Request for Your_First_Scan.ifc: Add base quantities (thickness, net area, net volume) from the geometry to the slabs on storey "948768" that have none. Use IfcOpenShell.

First a look at what the model holds.

```python
import ifcopenshell
import ifcopenshell.util.element
import ifcopenshell.util.unit

model = ifcopenshell.open("Your_First_Scan.ifc")
print(model.schema)
for unit_type in ("LENGTHUNIT", "AREAUNIT", "VOLUMEUNIT"):
    print(unit_type, ifcopenshell.util.unit.calculate_unit_scale(model, unit_type))
storey = next(s for s in model.by_type("IfcBuildingStorey") if s.Name == "948768")
slabs = [e for e in ifcopenshell.util.element.get_decomposition(storey) if e.is_a("IfcSlab")]
for e in sorted(slabs, key=lambda e: e.id()):
    print(e.id(), e.is_a(), e.Name, list(ifcopenshell.util.element.get_psets(e, qtos_only=True)), sep=" | ")
```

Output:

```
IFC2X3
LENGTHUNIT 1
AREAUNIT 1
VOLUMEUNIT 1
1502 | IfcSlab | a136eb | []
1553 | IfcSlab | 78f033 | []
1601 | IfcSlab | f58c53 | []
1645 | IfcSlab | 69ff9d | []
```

```python
import ifcopenshell
import ifcopenshell.api.pset
import ifcopenshell.geom
import ifcopenshell.util.element
import ifcopenshell.util.shape
import ifcopenshell.util.unit

model = ifcopenshell.open("Your_First_Scan.ifc")
unit_scale = ifcopenshell.util.unit.calculate_unit_scale(model)
area_scale = ifcopenshell.util.unit.calculate_unit_scale(model, "AREAUNIT")
volume_scale = ifcopenshell.util.unit.calculate_unit_scale(model, "VOLUMEUNIT")
settings = ifcopenshell.geom.settings()

storey = next(s for s in model.by_type("IfcBuildingStorey") if s.Name == "948768")
slabs = [e for e in ifcopenshell.util.element.get_decomposition(storey) if e.is_a("IfcSlab")]

for e in sorted(slabs, key=lambda e: e.id()):
    if ifcopenshell.util.element.get_psets(e, qtos_only=True, should_inherit=False):
        continue
    # Geometry comes back in metres, in the element's own axes.
    shape = ifcopenshell.geom.create_shape(settings, e)
    values = {
        "Width": ifcopenshell.util.shape.get_z(shape.geometry) / unit_scale,
        "NetArea": ifcopenshell.util.shape.get_footprint_area(shape.geometry) / area_scale,
        "NetVolume": ifcopenshell.util.shape.get_volume(shape.geometry) / volume_scale,
    }
    qto = ifcopenshell.api.pset.add_qto(model, product=e, name="BaseQuantities")
    ifcopenshell.api.pset.edit_qto(model, qto=qto, properties=values)
    print(e.id(), {k: round(v, 3) for k, v in values.items()})

model.write("Your_First_Scan_rev.ifc")
```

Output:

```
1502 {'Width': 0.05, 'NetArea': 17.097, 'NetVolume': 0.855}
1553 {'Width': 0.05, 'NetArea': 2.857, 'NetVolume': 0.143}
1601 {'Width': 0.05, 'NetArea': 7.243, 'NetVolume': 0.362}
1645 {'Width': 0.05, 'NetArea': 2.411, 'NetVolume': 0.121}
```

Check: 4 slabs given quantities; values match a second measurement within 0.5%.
